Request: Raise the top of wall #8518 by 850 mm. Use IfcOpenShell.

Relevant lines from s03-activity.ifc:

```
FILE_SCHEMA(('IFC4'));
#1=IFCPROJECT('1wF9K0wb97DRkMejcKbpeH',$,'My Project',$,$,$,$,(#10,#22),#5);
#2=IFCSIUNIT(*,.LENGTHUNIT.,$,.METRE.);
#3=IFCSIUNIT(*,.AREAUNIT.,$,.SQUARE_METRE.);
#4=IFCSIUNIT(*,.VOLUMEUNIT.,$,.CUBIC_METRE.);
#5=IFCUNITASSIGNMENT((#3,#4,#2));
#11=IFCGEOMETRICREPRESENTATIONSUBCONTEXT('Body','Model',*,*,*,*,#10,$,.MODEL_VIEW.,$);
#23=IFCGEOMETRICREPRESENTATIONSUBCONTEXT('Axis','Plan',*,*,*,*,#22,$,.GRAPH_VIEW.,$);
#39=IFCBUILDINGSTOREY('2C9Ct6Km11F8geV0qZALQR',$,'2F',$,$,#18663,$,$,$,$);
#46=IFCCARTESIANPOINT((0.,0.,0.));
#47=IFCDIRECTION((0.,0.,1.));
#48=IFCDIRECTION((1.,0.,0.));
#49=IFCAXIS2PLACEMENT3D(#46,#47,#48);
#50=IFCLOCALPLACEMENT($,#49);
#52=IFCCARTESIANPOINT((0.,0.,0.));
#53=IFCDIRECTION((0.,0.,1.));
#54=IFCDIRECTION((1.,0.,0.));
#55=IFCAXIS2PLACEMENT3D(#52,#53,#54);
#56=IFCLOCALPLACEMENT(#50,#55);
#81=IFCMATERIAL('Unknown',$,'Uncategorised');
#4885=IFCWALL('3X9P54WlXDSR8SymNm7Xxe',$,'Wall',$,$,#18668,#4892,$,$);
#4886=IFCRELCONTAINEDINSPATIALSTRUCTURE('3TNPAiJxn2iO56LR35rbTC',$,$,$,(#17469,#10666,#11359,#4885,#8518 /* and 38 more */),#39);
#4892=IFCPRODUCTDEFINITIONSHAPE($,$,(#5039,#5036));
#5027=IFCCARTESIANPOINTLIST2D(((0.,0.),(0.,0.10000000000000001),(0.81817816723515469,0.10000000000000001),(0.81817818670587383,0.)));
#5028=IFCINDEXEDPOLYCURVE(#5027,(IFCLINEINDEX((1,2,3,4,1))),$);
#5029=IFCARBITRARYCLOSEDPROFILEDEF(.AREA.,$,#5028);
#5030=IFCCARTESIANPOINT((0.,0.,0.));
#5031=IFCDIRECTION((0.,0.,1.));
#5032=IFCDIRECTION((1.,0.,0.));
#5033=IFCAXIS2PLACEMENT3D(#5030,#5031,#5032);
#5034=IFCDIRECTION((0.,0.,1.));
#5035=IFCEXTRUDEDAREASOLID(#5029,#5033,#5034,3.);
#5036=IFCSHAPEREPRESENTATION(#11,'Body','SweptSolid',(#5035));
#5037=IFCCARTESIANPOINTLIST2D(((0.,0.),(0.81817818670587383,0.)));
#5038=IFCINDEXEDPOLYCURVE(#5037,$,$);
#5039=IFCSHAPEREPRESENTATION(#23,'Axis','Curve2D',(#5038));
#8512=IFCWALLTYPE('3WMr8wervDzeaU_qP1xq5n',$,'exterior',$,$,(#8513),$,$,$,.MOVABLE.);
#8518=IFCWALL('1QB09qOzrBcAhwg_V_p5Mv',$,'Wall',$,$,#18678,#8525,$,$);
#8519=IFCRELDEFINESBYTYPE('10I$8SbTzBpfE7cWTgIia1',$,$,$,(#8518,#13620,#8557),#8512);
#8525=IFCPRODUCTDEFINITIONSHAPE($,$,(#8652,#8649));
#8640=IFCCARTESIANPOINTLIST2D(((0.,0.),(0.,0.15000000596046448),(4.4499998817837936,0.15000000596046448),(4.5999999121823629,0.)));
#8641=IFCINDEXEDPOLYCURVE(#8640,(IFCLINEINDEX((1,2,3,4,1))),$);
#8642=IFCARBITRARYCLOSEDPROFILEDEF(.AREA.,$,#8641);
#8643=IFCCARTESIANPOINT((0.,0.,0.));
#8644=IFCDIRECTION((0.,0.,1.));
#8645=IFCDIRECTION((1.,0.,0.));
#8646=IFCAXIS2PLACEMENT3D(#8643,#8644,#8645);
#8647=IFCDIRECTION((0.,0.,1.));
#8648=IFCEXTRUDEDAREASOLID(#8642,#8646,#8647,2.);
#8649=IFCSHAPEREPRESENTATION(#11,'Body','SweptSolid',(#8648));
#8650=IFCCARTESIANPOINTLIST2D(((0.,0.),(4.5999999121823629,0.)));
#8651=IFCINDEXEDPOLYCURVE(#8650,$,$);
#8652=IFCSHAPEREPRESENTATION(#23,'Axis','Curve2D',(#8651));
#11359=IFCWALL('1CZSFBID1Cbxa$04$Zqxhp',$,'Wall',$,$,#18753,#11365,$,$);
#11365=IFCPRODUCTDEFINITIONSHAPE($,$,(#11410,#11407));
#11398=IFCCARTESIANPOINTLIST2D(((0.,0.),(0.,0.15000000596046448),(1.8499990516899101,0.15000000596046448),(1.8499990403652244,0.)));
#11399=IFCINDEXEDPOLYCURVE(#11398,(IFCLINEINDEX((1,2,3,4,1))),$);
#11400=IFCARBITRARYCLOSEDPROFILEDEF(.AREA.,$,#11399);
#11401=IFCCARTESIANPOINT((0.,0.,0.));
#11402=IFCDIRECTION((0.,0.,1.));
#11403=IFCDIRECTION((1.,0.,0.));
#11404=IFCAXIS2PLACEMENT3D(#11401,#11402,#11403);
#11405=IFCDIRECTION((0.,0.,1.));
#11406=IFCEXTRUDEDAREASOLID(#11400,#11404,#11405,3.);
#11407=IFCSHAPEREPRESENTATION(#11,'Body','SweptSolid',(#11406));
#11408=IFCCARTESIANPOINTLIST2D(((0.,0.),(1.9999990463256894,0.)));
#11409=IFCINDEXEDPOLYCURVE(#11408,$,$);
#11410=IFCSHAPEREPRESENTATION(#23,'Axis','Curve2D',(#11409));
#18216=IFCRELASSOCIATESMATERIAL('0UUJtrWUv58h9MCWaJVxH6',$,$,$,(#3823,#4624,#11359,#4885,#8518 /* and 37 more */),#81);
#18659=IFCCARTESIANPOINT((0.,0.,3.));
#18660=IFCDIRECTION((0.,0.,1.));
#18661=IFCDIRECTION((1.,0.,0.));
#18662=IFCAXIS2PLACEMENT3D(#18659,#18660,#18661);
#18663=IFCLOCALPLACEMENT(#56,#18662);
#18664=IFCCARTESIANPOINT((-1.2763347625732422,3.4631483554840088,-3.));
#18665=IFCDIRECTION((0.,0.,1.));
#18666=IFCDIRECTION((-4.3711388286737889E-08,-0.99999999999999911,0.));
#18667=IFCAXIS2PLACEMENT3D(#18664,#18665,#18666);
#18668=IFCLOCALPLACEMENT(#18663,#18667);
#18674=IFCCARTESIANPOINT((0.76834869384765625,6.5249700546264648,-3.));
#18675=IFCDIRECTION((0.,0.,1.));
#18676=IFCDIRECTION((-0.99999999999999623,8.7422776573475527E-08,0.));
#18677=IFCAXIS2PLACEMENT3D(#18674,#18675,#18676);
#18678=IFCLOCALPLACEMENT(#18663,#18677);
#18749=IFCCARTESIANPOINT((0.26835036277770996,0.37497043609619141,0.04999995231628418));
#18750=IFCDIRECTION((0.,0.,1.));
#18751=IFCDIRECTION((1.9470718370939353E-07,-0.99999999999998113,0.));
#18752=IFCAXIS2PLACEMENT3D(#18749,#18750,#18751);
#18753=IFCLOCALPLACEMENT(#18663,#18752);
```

```python
import ifcopenshell
import ifcopenshell.geom
import ifcopenshell.util.representation
import ifcopenshell.util.shape
import ifcopenshell.util.unit

model = ifcopenshell.open("s03-activity.ifc")
unit_scale = ifcopenshell.util.unit.calculate_unit_scale(model)
settings = ifcopenshell.geom.settings()


def volume(element):
    """Net volume in cubic metres, openings subtracted."""
    shape = ifcopenshell.geom.create_shape(settings, element)
    return ifcopenshell.util.shape.get_volume(shape.geometry)


wall = model.by_guid("1QB09qOzrBcAhwg_V_p5Mv")
before = volume(wall)

body = ifcopenshell.util.representation.get_representation(wall, "Model", "Body")
solid = body.Items[0]
old_height = solid.Depth
solid.Depth += 0.85 / unit_scale
after = volume(wall)

print(f"height {old_height:g} -> {solid.Depth:g}, volume {before:.3f} -> {after:.3f} m3")

model.write("s03-activity_v2.ifc")
```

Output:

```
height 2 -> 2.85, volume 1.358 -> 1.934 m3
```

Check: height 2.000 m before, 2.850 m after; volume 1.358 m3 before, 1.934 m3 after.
